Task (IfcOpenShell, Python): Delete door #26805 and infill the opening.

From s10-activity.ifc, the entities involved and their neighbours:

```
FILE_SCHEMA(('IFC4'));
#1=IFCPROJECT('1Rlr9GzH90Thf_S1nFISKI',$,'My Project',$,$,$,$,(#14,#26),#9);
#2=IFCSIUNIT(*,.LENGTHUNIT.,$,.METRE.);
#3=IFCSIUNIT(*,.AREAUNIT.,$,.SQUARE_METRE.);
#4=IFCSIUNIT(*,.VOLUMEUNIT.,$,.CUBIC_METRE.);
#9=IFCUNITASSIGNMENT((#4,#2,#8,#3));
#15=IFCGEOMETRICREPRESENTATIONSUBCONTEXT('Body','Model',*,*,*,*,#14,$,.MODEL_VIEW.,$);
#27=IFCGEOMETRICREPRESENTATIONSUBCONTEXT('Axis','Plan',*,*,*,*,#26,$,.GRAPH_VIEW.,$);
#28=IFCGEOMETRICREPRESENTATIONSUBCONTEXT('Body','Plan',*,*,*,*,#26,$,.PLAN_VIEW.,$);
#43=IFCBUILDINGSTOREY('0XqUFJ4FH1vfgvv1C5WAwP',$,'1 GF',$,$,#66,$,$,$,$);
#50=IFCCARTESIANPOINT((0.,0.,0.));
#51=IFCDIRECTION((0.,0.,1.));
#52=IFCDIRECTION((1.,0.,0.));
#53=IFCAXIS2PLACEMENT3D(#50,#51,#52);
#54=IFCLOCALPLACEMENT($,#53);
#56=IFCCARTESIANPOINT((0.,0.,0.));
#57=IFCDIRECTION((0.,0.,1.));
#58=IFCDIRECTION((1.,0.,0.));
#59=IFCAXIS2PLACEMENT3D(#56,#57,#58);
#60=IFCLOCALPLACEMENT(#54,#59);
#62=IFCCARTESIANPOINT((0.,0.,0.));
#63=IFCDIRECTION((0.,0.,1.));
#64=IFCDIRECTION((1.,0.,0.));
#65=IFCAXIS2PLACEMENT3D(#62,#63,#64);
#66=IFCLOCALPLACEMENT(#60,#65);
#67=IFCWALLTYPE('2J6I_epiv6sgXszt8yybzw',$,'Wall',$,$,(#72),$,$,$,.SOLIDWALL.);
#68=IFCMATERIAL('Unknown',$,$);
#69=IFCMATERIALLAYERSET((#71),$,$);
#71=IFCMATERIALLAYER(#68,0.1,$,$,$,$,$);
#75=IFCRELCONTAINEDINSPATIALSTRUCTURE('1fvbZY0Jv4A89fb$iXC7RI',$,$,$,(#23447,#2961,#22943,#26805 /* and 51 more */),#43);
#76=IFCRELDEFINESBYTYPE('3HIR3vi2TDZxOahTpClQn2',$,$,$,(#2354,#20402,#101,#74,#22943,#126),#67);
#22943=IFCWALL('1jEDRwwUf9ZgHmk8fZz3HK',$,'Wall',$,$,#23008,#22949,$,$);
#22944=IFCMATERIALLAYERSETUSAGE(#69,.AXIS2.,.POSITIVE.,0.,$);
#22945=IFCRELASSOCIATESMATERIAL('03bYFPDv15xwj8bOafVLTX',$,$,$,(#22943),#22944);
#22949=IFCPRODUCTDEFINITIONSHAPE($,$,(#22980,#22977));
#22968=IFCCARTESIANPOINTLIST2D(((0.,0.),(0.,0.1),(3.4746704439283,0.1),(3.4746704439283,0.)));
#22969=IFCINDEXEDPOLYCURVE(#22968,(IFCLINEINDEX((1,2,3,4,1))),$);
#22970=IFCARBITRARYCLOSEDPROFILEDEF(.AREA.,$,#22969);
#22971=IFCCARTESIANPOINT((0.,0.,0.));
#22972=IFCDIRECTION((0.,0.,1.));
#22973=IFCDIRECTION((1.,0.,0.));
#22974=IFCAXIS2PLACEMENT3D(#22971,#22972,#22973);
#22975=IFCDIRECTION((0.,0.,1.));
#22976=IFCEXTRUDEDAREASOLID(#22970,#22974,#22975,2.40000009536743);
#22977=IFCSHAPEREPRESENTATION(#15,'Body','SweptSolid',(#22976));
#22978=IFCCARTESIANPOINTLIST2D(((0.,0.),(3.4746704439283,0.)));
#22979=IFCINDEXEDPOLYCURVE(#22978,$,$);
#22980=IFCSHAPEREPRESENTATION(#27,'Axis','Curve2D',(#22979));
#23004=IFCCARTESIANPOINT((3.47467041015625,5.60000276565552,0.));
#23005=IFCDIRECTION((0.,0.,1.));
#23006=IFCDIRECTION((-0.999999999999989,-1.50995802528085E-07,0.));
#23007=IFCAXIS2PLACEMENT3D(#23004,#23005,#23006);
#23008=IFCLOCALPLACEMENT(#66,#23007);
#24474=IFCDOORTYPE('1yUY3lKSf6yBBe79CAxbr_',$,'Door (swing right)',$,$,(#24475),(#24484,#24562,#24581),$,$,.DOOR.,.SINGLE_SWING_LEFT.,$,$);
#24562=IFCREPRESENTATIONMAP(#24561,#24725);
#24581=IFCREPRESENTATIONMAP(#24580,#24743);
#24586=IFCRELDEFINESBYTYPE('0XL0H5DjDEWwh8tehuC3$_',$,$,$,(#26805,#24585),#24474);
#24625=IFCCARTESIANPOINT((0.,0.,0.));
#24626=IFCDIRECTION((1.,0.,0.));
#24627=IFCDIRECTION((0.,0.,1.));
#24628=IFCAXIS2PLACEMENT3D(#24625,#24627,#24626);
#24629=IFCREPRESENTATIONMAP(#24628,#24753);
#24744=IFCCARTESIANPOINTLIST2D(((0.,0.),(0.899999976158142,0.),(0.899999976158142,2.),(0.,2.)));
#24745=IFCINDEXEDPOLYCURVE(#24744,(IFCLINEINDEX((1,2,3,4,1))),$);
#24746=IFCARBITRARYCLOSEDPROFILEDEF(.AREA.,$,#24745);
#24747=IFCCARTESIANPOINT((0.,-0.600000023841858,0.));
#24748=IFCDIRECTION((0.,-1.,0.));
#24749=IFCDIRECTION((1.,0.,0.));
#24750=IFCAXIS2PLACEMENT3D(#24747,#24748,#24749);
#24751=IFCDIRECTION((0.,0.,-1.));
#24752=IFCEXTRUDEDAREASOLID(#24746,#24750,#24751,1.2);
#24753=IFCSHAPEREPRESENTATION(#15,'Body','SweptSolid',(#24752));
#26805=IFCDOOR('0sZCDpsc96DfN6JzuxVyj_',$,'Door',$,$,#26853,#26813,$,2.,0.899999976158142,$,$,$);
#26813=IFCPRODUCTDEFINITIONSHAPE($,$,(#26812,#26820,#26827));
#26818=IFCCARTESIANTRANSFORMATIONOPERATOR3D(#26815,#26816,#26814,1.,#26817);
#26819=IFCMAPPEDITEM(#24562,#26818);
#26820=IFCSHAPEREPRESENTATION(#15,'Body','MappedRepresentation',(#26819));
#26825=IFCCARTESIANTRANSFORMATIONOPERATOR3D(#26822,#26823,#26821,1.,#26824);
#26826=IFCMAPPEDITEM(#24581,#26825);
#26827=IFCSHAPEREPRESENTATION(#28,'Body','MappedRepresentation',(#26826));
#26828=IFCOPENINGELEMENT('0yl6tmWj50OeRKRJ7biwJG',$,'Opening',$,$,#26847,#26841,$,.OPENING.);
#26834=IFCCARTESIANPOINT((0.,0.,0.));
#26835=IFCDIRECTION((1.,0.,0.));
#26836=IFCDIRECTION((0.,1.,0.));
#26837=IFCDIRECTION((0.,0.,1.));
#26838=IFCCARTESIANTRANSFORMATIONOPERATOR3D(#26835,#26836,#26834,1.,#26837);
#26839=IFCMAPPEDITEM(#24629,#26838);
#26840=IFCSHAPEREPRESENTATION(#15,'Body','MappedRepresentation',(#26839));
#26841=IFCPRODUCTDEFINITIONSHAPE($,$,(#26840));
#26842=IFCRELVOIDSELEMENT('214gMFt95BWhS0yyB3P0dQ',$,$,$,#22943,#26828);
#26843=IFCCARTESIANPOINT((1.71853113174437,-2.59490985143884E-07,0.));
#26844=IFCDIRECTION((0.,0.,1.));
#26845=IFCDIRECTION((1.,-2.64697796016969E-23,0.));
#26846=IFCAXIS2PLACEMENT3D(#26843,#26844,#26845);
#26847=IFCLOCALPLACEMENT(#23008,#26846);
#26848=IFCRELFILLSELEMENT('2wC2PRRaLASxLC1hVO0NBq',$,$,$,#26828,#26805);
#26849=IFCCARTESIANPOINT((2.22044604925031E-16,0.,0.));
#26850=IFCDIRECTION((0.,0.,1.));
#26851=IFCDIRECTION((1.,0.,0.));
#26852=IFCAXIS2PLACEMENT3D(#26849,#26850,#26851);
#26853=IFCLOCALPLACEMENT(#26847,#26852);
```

```python
import ifcopenshell
import ifcopenshell.api.feature
import ifcopenshell.api.root
import ifcopenshell.geom
import ifcopenshell.util.shape

model = ifcopenshell.open("s10-activity.ifc")
settings = ifcopenshell.geom.settings()


def volume(element):
    """Net volume in cubic metres, openings subtracted."""
    shape = ifcopenshell.geom.create_shape(settings, element)
    return ifcopenshell.util.shape.get_volume(shape.geometry)


door = model.by_guid("0sZCDpsc96DfN6JzuxVyj_")
opening = door.FillsVoids[0].RelatingOpeningElement
wall = opening.VoidsElements[0].RelatingBuildingElement
before = volume(wall)

ifcopenshell.api.root.remove_product(model, product=door)
ifcopenshell.api.feature.remove_feature(model, feature=opening)

after = volume(wall)

print(f"wall volume {before:.3f} -> {after:.3f} m3")

model.write("s10-activity-out.ifc")
```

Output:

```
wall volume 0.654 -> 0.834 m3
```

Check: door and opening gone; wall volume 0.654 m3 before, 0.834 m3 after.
